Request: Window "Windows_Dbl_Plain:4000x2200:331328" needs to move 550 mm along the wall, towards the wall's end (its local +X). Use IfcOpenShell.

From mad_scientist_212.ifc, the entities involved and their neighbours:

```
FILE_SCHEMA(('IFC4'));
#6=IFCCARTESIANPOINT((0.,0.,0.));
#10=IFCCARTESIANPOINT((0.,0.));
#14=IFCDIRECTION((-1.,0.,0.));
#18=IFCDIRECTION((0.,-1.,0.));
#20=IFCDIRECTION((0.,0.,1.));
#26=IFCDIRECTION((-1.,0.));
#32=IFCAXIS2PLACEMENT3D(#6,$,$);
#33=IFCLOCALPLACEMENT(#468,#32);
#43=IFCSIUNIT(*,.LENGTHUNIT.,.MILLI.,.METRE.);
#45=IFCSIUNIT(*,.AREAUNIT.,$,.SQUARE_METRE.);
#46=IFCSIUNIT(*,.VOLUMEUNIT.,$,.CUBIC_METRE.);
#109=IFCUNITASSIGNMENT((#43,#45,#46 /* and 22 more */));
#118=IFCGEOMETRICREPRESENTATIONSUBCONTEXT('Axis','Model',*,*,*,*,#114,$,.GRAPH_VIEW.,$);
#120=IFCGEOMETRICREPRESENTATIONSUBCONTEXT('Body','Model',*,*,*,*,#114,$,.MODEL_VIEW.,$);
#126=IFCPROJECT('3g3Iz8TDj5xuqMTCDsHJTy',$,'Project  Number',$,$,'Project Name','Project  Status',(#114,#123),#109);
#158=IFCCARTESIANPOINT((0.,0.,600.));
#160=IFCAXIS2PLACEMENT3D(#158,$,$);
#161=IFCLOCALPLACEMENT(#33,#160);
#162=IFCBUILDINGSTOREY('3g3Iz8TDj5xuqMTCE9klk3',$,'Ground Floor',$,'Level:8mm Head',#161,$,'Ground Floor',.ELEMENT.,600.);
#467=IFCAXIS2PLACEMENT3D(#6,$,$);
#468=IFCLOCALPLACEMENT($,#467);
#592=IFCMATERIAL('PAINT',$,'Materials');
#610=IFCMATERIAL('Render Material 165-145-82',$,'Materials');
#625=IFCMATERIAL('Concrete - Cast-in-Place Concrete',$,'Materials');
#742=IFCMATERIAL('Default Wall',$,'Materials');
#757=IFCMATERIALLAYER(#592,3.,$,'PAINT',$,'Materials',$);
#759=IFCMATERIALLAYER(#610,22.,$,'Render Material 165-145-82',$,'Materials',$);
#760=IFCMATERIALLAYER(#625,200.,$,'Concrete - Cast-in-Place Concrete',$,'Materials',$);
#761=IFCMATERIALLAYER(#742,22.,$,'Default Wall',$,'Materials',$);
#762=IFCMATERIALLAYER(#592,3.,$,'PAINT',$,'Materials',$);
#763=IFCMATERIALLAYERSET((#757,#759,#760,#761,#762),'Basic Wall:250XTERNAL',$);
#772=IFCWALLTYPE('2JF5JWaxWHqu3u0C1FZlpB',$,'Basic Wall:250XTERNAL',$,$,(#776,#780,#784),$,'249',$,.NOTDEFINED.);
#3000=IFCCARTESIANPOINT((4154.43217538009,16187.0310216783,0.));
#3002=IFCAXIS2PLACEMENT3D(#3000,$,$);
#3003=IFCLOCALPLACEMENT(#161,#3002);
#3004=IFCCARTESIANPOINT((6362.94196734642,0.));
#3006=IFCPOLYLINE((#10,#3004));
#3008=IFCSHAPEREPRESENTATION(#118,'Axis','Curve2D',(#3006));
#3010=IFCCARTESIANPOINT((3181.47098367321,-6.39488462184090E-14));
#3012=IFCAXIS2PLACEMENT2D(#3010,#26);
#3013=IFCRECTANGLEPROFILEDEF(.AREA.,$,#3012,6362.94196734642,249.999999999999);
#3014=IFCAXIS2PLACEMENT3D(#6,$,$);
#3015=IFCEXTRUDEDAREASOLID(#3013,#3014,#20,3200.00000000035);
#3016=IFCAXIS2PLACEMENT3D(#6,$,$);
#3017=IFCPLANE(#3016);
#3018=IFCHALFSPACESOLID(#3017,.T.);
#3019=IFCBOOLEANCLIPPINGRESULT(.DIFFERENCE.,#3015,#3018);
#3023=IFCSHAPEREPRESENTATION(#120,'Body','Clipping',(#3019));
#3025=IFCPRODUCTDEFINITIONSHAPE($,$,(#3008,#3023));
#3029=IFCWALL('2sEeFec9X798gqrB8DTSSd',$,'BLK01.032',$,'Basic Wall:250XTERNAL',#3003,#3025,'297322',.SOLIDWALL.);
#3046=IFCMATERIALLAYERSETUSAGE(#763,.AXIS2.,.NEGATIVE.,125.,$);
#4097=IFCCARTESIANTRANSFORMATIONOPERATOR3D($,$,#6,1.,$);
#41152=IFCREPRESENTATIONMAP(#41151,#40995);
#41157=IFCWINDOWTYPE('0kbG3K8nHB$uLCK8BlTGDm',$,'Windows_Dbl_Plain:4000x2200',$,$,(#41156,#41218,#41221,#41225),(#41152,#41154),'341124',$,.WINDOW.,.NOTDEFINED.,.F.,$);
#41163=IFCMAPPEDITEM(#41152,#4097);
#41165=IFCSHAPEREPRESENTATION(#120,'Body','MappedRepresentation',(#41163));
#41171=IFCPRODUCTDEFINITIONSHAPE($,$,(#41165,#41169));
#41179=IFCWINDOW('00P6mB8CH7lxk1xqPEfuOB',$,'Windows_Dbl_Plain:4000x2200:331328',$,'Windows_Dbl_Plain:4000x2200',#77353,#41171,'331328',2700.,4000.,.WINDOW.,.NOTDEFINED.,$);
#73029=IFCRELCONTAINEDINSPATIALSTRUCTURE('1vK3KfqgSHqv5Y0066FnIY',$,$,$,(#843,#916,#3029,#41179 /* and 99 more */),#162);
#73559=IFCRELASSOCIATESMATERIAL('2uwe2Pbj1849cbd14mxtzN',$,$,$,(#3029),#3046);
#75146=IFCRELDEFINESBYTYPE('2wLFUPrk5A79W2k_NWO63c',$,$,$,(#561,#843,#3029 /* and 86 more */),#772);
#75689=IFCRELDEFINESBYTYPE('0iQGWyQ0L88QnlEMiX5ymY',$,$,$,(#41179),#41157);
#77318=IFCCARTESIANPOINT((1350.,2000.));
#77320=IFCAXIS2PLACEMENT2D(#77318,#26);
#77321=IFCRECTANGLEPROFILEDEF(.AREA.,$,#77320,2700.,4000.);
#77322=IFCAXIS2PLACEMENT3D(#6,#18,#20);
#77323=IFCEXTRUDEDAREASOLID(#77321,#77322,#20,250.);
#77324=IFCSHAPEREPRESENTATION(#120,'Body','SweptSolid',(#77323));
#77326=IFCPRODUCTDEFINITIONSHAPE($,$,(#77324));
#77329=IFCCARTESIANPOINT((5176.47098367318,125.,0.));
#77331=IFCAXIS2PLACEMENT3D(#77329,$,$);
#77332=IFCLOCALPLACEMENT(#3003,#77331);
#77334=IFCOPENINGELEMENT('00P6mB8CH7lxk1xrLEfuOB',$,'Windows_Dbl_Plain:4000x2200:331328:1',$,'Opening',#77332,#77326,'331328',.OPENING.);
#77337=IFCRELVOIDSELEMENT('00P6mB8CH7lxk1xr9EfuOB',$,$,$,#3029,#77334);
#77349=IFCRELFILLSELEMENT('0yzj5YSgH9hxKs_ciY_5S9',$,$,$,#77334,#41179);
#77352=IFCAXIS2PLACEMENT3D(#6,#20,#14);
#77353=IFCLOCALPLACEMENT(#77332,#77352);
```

```python
import ifcopenshell
import ifcopenshell.api.geometry
import ifcopenshell.util.placement
import ifcopenshell.util.unit

model = ifcopenshell.open("mad_scientist_212.ifc")
unit_scale = ifcopenshell.util.unit.calculate_unit_scale(model)

window = model.by_guid("00P6mB8CH7lxk1xqPEfuOB")
opening = window.FillsVoids[0].RelatingOpeningElement
wall = opening.VoidsElements[0].RelatingBuildingElement

wall_matrix = ifcopenshell.util.placement.get_local_placement(wall.ObjectPlacement)
shift = wall_matrix[:3, 0] * 0.55 / unit_scale
before = ifcopenshell.util.placement.get_local_placement(window.ObjectPlacement)[:3, 3].copy()

# The window is placed relative to its opening, so it follows when the opening moves.
matrix = ifcopenshell.util.placement.get_local_placement(opening.ObjectPlacement)
matrix[:3, 3] += shift
ifcopenshell.api.geometry.edit_object_placement(
    model, product=opening, matrix=matrix, is_si=False, should_transform_children=True
)

after = ifcopenshell.util.placement.get_local_placement(window.ObjectPlacement)[:3, 3]
print("window moved by", (after - before).round(3) + 0.0)

model.write("mad_scientist_212-out.ifc")
```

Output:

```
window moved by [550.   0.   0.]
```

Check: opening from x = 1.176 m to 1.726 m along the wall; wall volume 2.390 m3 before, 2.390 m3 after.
